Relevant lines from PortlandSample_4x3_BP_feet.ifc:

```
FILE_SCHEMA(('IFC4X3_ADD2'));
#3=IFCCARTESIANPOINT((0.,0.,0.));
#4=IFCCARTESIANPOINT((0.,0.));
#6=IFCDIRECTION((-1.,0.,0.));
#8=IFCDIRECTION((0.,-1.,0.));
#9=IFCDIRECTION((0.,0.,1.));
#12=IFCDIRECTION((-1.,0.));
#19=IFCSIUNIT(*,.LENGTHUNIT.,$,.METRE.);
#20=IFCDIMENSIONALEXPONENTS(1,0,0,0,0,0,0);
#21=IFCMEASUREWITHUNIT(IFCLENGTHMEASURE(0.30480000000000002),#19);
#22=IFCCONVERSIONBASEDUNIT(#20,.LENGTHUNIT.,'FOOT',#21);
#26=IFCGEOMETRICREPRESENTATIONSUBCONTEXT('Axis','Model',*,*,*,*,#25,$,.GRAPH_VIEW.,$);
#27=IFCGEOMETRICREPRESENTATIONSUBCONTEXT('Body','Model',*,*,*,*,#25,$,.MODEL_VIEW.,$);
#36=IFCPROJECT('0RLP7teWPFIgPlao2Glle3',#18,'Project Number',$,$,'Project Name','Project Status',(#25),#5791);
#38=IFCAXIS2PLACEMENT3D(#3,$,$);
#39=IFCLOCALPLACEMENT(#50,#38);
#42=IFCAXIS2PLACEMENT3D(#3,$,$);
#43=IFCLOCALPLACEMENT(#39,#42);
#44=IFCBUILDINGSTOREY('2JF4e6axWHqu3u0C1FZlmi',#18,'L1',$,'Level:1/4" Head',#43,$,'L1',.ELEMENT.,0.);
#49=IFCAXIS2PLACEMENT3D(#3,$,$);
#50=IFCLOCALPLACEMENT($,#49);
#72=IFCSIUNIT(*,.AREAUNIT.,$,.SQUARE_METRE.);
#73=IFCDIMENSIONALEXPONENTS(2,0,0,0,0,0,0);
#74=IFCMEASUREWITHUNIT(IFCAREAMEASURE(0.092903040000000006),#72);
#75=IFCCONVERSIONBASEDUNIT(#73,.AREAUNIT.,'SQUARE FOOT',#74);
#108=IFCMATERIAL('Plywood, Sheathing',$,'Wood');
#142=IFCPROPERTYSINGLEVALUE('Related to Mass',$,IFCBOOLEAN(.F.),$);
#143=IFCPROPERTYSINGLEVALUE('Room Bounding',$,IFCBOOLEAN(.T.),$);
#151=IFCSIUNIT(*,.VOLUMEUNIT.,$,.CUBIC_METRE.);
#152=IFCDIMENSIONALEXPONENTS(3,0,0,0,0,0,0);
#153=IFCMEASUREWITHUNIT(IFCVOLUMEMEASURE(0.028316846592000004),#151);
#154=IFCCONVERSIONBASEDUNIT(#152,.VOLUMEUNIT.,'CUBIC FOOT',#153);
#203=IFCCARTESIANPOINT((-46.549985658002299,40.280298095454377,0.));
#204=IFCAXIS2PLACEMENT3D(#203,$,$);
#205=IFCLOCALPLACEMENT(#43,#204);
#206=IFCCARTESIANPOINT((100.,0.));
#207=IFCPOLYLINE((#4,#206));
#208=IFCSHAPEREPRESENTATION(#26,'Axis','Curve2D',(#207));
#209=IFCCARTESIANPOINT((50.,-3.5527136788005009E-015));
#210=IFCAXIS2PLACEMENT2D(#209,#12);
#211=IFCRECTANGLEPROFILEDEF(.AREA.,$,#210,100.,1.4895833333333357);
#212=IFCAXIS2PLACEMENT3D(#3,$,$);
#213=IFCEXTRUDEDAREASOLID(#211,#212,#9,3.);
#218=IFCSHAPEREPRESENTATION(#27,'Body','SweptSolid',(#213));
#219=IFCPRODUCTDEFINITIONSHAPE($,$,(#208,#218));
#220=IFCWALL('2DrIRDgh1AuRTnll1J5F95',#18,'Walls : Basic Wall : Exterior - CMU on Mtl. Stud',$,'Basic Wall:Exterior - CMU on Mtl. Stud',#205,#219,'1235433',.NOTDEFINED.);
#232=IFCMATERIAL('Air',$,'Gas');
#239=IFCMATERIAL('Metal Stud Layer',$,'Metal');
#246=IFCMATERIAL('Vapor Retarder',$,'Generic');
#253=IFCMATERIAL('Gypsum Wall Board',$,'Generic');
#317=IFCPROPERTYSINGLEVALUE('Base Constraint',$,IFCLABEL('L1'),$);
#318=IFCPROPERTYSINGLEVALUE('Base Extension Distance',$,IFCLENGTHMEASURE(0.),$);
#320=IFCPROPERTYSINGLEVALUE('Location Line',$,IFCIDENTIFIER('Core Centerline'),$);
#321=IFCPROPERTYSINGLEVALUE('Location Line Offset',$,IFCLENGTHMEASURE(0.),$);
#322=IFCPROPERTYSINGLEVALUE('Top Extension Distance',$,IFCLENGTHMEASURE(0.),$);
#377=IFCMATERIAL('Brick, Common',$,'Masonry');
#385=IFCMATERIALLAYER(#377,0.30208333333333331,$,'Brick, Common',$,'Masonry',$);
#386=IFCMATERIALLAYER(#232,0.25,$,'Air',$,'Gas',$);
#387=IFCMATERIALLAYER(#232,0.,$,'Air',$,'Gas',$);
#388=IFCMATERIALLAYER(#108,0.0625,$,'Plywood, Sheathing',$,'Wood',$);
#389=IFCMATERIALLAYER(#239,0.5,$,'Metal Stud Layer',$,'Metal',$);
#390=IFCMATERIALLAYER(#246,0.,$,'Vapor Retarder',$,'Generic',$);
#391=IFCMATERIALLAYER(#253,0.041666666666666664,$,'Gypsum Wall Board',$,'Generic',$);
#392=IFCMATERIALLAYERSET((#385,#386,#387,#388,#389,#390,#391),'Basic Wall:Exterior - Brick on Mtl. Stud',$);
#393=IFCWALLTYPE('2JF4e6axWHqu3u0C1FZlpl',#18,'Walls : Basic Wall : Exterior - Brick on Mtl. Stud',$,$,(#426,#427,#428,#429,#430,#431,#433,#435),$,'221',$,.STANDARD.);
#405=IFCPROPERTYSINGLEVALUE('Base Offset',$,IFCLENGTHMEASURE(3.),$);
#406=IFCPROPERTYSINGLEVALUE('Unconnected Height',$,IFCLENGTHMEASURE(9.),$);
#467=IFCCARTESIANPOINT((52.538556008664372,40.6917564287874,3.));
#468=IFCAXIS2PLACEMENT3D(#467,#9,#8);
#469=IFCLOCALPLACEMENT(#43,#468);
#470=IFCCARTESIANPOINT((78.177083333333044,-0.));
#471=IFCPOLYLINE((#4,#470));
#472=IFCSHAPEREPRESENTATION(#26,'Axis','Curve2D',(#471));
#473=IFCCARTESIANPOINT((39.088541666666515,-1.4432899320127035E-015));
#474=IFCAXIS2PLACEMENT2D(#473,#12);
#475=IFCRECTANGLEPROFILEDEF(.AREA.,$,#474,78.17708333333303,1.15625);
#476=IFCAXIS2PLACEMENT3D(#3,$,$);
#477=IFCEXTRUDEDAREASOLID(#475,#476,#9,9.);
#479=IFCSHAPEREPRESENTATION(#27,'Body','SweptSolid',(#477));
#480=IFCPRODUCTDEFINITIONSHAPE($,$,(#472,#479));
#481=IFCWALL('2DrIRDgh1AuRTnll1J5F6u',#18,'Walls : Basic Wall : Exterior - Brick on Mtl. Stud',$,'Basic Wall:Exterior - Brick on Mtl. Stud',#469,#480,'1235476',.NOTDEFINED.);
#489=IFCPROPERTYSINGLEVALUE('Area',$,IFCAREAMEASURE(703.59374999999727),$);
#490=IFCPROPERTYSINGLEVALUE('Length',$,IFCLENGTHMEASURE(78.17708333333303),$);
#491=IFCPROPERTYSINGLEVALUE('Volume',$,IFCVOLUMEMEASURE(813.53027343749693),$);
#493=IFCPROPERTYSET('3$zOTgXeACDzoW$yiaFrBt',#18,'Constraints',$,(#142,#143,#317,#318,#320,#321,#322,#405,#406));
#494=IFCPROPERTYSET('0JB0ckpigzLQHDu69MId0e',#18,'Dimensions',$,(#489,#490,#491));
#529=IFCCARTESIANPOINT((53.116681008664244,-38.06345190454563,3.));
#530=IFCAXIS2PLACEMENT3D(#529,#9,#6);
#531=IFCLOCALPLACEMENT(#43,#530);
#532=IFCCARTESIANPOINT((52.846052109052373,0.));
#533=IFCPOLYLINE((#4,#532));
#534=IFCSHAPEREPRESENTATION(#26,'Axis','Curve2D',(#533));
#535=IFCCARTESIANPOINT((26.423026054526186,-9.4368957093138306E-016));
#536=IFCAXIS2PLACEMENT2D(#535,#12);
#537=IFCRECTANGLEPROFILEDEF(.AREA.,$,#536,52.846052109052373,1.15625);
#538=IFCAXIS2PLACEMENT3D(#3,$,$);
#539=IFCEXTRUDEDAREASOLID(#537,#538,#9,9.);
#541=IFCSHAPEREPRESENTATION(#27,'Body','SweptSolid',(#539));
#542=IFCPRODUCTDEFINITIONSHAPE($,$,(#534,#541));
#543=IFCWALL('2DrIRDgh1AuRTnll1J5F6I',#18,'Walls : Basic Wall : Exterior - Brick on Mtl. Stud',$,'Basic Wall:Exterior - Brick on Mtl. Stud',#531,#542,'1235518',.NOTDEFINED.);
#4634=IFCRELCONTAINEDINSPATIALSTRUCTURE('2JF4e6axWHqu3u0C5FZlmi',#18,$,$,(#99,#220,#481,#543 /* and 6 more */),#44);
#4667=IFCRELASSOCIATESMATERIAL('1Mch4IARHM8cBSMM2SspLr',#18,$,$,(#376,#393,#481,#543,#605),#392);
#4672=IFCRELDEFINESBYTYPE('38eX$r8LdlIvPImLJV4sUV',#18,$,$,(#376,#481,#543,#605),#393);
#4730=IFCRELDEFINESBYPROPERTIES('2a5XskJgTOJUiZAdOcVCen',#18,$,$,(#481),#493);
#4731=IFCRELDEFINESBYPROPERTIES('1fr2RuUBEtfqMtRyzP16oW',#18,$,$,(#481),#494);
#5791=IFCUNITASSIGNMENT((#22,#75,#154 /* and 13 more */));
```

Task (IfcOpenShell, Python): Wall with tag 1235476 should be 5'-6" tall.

```python
import ifcopenshell
import ifcopenshell.api.pset
import ifcopenshell.geom
import ifcopenshell.util.element
import ifcopenshell.util.representation
import ifcopenshell.util.shape
import ifcopenshell.util.unit

model = ifcopenshell.open("PortlandSample_4x3_BP_feet.ifc")
unit_scale = ifcopenshell.util.unit.calculate_unit_scale(model)
area_scale = ifcopenshell.util.unit.calculate_unit_scale(model, "AREAUNIT")
volume_scale = ifcopenshell.util.unit.calculate_unit_scale(model, "VOLUMEUNIT")
settings = ifcopenshell.geom.settings()


def volume(element):
    """Net volume in cubic metres, openings subtracted."""
    shape = ifcopenshell.geom.create_shape(settings, element)
    return ifcopenshell.util.shape.get_volume(shape.geometry)


wall = model.by_guid("2DrIRDgh1AuRTnll1J5F6u")
before = volume(wall)

body = ifcopenshell.util.representation.get_representation(wall, "Model", "Body")
solid = body.Items[0]
old_height = solid.Depth
solid.Depth = 66 * 0.0254 / unit_scale
after = volume(wall)
thickness = 0.3524  # wall thickness in metres

# Update the stored height, areas and volumes.
pset = model.by_id(ifcopenshell.util.element.get_pset(wall, "Constraints", should_inherit=False)["id"])
ifcopenshell.api.pset.edit_pset(model, pset=pset, properties={
    "Unconnected Height": model.create_entity("IfcLengthMeasure", solid.Depth),
})
pset = model.by_id(ifcopenshell.util.element.get_pset(wall, "Dimensions", should_inherit=False)["id"])
ifcopenshell.api.pset.edit_pset(model, pset=pset, properties={
    "Area": model.create_entity("IfcAreaMeasure", after / thickness / area_scale),
    "Volume": model.create_entity("IfcVolumeMeasure", after / volume_scale),
})

print(f"height {old_height:g} -> {solid.Depth:g}, volume {before:.3f} -> {after:.3f} m3")

model.write("PortlandSample_4x3_BP_feet_updated.ifc")
```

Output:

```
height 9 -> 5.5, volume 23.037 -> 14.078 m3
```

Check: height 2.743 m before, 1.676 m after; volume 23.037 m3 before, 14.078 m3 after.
